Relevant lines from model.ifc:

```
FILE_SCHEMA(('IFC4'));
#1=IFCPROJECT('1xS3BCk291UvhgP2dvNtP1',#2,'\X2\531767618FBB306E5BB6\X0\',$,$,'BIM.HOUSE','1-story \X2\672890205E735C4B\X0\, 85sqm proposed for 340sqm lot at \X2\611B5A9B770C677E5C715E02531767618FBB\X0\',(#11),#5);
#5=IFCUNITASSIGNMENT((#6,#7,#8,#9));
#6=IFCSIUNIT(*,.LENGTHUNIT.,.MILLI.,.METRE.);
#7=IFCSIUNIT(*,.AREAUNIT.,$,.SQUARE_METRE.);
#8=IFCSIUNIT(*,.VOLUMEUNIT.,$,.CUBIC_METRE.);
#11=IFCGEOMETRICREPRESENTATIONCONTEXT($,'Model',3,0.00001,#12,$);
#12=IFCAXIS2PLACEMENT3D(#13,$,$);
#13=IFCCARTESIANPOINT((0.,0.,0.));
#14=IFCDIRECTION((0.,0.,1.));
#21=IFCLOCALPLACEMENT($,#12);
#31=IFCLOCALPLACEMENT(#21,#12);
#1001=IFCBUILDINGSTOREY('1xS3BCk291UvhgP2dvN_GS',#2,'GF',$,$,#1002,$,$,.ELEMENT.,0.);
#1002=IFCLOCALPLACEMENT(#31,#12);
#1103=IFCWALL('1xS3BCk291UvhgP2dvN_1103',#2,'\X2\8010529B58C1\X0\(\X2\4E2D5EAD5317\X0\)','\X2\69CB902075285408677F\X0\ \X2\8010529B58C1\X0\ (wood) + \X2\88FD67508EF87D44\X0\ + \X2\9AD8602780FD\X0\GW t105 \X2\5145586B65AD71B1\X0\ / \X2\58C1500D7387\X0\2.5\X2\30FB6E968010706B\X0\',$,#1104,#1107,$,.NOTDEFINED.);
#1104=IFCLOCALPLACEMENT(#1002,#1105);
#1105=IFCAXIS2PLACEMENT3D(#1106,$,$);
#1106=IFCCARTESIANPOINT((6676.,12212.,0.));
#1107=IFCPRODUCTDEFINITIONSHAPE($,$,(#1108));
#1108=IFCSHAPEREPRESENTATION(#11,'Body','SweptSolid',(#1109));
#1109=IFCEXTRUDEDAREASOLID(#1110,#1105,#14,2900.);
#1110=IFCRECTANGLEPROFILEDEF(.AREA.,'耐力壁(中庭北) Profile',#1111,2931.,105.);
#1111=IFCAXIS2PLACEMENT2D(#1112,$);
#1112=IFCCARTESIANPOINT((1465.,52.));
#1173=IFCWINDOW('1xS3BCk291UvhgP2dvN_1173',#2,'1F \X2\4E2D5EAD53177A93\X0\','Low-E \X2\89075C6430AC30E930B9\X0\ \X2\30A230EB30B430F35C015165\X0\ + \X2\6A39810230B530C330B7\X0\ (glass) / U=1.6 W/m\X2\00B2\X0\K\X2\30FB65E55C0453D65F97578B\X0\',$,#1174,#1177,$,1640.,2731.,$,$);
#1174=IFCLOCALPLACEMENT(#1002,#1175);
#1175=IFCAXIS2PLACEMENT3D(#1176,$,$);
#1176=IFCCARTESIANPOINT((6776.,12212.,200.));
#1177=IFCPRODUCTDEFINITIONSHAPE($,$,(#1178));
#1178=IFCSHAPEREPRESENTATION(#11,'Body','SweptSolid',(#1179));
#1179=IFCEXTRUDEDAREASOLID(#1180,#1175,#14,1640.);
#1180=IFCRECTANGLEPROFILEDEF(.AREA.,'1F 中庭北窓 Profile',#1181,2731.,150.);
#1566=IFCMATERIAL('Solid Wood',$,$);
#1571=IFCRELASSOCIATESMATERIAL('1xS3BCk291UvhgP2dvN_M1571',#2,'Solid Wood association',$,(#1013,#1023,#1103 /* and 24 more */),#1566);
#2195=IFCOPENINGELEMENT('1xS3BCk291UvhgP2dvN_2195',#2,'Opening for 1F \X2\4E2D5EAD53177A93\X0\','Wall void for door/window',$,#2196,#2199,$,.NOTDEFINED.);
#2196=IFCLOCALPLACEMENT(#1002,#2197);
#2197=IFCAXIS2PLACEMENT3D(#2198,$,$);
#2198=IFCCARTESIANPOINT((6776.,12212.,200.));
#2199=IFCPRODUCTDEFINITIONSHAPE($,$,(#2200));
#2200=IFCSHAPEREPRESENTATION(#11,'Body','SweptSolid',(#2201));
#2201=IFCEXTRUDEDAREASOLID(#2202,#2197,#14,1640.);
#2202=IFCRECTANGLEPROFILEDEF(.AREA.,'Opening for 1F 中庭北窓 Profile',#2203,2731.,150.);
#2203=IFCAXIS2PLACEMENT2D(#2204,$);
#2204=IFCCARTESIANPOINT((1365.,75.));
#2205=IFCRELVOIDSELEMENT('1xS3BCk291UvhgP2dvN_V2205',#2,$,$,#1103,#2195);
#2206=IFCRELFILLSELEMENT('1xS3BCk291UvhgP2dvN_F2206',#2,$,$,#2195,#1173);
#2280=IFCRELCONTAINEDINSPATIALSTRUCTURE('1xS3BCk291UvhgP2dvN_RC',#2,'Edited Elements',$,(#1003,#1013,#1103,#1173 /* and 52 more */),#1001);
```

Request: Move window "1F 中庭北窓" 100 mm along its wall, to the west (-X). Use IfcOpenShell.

```python
import ifcopenshell
import ifcopenshell.api.geometry
import ifcopenshell.util.placement
import ifcopenshell.util.unit

model = ifcopenshell.open("model.ifc")
unit_scale = ifcopenshell.util.unit.calculate_unit_scale(model)

window = model.by_guid("1xS3BCk291UvhgP2dvN_1173")
opening = window.FillsVoids[0].RelatingOpeningElement
wall = opening.VoidsElements[0].RelatingBuildingElement

wall_matrix = ifcopenshell.util.placement.get_local_placement(wall.ObjectPlacement)
shift = wall_matrix[:3, 0] * -0.1 / unit_scale
before = ifcopenshell.util.placement.get_local_placement(window.ObjectPlacement)[:3, 3].copy()

# The window is not placed relative to its opening, so move both.
for product in (opening, window):
    matrix = ifcopenshell.util.placement.get_local_placement(product.ObjectPlacement)
    matrix[:3, 3] += shift
    ifcopenshell.api.geometry.edit_object_placement(model, product=product, matrix=matrix, is_si=False)

after = ifcopenshell.util.placement.get_local_placement(window.ObjectPlacement)[:3, 3]
print("window moved by", (after - before).round(3) + 0.0)

model.write("model_rev.ifc")
```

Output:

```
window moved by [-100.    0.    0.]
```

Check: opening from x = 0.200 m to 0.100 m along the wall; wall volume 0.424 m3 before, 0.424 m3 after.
